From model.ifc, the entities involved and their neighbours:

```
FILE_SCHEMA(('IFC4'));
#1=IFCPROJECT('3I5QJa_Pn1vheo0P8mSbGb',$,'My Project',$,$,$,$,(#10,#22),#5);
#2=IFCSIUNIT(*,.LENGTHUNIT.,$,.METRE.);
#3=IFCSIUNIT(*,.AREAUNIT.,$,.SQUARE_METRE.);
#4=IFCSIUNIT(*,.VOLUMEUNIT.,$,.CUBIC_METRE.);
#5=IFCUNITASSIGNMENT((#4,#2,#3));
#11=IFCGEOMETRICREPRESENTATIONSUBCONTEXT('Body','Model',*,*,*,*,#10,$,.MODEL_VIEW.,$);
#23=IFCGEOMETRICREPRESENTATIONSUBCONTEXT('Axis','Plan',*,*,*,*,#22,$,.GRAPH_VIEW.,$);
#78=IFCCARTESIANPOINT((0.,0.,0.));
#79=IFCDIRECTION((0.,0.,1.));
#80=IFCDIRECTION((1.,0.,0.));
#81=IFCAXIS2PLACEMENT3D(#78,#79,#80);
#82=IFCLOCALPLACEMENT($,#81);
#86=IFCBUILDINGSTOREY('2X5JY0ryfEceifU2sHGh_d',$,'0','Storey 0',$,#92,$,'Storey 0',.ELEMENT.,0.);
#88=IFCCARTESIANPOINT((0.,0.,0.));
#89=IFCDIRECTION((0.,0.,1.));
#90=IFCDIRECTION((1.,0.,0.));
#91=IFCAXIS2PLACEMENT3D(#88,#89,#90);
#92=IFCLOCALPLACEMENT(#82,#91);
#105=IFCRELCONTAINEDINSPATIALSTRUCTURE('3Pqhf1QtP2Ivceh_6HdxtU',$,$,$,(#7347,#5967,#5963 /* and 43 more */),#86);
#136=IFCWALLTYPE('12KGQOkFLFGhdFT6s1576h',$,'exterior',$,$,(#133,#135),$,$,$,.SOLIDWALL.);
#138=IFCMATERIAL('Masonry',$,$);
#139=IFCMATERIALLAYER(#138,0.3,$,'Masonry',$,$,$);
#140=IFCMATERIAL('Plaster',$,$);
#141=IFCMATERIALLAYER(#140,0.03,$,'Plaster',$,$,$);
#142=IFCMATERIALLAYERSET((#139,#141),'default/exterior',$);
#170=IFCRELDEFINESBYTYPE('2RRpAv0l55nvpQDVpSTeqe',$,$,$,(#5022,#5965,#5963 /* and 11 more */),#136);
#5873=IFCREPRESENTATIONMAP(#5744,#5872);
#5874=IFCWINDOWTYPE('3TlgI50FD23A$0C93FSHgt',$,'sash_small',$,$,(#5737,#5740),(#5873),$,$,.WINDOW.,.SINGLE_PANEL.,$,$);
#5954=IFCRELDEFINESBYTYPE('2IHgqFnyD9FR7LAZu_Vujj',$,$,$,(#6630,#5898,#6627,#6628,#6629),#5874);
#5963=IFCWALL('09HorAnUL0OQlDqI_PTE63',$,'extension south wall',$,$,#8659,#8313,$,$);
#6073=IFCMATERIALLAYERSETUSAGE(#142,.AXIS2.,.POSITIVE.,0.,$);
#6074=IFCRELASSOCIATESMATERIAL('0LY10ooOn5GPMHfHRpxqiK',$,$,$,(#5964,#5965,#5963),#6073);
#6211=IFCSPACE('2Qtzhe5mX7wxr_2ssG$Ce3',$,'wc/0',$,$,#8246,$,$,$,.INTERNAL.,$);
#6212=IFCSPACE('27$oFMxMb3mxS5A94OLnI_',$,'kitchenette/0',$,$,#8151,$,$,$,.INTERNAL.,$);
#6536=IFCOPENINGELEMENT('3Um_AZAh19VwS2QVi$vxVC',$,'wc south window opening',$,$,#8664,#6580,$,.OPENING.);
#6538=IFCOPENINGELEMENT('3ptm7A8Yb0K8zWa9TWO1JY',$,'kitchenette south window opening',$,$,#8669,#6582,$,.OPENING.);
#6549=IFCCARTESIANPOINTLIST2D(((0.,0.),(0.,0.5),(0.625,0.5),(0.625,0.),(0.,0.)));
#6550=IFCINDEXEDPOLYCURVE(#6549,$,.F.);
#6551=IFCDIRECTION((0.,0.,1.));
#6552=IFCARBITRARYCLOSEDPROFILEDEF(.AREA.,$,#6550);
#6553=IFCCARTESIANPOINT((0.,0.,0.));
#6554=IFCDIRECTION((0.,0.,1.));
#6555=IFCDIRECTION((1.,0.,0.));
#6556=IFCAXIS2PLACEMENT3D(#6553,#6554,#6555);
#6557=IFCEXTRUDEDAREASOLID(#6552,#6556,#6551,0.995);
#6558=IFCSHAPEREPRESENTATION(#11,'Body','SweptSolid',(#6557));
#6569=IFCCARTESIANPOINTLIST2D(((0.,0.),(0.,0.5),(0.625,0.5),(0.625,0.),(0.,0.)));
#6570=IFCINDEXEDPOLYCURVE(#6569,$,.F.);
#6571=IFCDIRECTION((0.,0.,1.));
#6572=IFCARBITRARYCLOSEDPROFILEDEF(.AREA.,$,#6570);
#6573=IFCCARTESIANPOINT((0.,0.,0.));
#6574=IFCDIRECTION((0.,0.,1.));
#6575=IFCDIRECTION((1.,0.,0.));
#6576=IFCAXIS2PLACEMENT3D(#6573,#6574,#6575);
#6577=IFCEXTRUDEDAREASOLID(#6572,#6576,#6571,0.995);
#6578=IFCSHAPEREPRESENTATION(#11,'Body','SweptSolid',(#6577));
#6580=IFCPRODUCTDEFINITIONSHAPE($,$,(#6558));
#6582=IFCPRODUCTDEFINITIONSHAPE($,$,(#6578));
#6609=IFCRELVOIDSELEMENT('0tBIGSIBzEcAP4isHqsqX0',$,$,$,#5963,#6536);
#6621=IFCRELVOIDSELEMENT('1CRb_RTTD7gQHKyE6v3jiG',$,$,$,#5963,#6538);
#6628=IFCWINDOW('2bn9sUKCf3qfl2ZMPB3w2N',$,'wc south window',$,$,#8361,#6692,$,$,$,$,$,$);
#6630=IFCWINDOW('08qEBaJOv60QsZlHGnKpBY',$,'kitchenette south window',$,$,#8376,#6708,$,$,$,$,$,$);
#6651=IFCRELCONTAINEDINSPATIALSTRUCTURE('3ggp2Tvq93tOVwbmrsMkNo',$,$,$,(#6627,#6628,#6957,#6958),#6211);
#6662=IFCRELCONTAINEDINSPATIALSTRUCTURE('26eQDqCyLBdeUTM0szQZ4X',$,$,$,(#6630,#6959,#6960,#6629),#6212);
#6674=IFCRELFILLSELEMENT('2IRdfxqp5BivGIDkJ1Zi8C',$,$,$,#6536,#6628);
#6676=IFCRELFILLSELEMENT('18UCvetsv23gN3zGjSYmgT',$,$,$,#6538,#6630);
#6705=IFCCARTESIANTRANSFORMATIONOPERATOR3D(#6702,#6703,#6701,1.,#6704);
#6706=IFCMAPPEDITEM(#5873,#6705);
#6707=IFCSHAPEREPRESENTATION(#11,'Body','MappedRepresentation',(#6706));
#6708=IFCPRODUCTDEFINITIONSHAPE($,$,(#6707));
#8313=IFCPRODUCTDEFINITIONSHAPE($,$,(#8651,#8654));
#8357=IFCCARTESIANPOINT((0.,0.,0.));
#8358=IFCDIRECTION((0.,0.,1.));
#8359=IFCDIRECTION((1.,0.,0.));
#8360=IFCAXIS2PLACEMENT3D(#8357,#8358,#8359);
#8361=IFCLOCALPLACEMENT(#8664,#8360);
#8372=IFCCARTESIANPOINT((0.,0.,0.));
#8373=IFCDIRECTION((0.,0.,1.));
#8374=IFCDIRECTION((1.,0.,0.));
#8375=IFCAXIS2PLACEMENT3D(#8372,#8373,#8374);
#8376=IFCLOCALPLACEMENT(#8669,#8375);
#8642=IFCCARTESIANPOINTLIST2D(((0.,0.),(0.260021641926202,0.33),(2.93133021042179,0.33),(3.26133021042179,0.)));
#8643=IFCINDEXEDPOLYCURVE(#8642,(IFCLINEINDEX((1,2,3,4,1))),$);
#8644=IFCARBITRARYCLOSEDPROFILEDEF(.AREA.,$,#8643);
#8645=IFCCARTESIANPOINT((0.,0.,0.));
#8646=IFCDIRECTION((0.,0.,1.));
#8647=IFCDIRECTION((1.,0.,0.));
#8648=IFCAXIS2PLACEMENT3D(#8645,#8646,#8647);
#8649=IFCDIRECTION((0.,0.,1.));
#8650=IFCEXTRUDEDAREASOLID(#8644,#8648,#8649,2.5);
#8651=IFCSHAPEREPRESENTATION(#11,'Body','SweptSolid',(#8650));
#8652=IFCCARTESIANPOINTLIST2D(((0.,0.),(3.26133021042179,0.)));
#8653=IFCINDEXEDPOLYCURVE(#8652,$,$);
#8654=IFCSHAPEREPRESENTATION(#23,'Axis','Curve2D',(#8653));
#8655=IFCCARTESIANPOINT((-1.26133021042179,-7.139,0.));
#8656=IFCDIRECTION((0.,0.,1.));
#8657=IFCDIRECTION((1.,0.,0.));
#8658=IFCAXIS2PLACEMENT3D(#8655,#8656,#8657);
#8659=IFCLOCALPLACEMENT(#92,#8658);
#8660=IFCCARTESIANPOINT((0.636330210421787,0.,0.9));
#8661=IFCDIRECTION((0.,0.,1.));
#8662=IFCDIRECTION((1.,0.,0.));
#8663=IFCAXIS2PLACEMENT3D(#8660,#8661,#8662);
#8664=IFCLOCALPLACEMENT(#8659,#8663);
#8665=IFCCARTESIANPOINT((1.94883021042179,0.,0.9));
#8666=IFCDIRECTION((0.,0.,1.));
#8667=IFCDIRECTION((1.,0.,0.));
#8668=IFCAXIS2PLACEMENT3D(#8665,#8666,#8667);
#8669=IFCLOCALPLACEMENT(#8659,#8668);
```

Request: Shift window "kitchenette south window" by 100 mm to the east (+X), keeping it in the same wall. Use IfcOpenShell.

```python
import ifcopenshell
import ifcopenshell.api.geometry
import ifcopenshell.util.placement
import ifcopenshell.util.unit

model = ifcopenshell.open("model.ifc")
unit_scale = ifcopenshell.util.unit.calculate_unit_scale(model)

window = model.by_guid("08qEBaJOv60QsZlHGnKpBY")
opening = window.FillsVoids[0].RelatingOpeningElement
wall = opening.VoidsElements[0].RelatingBuildingElement

wall_matrix = ifcopenshell.util.placement.get_local_placement(wall.ObjectPlacement)
shift = wall_matrix[:3, 0] * 0.1 / unit_scale
before = ifcopenshell.util.placement.get_local_placement(window.ObjectPlacement)[:3, 3].copy()

# The window is placed relative to its opening, so it follows when the opening moves.
matrix = ifcopenshell.util.placement.get_local_placement(opening.ObjectPlacement)
matrix[:3, 3] += shift
ifcopenshell.api.geometry.edit_object_placement(
    model, product=opening, matrix=matrix, is_si=False, should_transform_children=True
)

after = ifcopenshell.util.placement.get_local_placement(window.ObjectPlacement)[:3, 3]
print("window moved by", (after - before).round(3) + 0.0)

model.write("model_rev.ifc")
```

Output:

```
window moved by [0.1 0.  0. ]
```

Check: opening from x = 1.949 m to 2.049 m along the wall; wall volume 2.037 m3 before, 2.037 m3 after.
